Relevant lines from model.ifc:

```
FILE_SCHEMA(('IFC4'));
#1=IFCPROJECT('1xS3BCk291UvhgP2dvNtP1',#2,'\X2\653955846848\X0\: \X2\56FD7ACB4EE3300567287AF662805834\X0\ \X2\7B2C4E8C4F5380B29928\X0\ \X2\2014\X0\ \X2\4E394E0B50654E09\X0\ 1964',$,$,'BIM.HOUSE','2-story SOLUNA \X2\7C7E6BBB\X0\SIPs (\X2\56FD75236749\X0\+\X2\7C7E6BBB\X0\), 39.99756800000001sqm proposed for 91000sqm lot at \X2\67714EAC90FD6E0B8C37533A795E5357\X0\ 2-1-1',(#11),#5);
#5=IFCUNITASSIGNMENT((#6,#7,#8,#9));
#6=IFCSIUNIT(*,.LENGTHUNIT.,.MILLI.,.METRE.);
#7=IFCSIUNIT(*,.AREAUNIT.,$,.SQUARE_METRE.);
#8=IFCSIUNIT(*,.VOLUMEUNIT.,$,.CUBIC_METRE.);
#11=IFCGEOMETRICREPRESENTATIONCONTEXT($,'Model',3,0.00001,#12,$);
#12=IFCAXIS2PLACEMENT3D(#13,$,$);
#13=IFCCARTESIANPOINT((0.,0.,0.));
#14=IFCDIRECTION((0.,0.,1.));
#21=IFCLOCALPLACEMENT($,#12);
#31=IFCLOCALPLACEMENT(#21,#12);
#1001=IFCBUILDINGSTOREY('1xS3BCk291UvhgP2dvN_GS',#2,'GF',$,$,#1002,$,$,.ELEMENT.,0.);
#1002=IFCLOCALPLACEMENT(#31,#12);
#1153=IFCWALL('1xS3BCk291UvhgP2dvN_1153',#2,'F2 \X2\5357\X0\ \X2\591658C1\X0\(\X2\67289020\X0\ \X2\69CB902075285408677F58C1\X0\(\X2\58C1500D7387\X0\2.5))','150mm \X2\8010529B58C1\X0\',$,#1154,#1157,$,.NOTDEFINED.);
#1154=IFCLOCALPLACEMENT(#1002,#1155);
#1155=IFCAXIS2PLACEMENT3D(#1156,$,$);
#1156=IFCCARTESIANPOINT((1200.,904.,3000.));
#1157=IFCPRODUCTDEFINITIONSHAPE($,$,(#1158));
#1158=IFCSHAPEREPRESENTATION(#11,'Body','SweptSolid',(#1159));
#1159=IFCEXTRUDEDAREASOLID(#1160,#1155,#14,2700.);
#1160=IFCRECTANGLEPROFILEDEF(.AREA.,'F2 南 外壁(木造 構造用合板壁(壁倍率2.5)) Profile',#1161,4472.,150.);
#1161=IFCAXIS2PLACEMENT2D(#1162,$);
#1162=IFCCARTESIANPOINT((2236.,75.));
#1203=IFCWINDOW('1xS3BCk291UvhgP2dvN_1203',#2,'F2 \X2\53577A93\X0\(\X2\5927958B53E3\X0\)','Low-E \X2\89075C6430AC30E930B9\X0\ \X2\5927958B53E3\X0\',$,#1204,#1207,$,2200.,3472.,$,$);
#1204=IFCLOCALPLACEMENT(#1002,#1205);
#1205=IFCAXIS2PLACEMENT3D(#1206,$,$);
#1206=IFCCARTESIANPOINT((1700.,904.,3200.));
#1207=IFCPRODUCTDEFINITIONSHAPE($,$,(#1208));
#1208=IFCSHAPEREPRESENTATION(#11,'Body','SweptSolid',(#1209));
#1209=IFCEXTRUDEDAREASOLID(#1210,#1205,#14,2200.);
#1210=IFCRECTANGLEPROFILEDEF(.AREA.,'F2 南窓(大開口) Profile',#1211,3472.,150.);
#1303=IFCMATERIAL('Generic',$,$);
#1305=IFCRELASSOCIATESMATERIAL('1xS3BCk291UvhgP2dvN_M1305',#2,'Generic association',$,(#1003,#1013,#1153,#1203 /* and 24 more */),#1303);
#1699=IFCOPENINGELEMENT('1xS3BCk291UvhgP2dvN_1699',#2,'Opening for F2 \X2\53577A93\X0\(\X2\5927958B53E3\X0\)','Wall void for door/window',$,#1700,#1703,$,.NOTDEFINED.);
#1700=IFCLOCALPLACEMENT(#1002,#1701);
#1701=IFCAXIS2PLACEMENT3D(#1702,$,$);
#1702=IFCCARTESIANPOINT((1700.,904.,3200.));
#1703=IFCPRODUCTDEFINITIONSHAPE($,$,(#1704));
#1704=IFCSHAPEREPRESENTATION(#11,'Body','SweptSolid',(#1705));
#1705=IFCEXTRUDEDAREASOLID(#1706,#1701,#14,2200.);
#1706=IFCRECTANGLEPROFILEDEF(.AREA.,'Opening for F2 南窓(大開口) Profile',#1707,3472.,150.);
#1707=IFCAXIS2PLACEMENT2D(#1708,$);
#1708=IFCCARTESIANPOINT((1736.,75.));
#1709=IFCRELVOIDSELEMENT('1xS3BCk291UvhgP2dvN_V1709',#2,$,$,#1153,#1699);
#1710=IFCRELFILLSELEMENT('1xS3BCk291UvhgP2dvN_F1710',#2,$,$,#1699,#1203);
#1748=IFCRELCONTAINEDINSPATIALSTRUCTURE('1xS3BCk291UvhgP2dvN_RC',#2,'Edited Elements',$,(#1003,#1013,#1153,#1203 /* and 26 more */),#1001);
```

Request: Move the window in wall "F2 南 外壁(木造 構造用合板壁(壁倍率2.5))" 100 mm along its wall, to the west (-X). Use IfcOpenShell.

```python
import ifcopenshell
import ifcopenshell.api.geometry
import ifcopenshell.util.placement
import ifcopenshell.util.unit

model = ifcopenshell.open("model.ifc")
unit_scale = ifcopenshell.util.unit.calculate_unit_scale(model)

window = model.by_guid("1xS3BCk291UvhgP2dvN_1203")
opening = window.FillsVoids[0].RelatingOpeningElement
wall = opening.VoidsElements[0].RelatingBuildingElement

wall_matrix = ifcopenshell.util.placement.get_local_placement(wall.ObjectPlacement)
shift = wall_matrix[:3, 0] * -0.1 / unit_scale
before = ifcopenshell.util.placement.get_local_placement(window.ObjectPlacement)[:3, 3].copy()

# The window is not placed relative to its opening, so move both.
for product in (opening, window):
    matrix = ifcopenshell.util.placement.get_local_placement(product.ObjectPlacement)
    matrix[:3, 3] += shift
    ifcopenshell.api.geometry.edit_object_placement(model, product=product, matrix=matrix, is_si=False)

after = ifcopenshell.util.placement.get_local_placement(window.ObjectPlacement)[:3, 3]
print("window moved by", (after - before).round(3) + 0.0)

model.write("model_edited.ifc")
```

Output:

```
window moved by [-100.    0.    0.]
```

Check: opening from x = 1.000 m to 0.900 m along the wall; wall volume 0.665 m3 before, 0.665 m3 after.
